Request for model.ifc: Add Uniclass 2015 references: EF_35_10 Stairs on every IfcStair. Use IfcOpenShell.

First a look at what the model holds.

```python
import ifcopenshell

model = ifcopenshell.open("model.ifc")
print(model.schema)
print("classifications:", [c.Name for c in model.by_type("IfcClassification")])
for ifc_class in ("IfcDoor", "IfcRoof", "IfcStair", "IfcWall", "IfcWindow"):
    print(ifc_class, len(model.by_type(ifc_class)))
```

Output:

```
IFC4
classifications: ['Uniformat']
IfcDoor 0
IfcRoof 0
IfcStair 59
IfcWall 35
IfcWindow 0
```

```python
import ifcopenshell
import ifcopenshell.api.classification

model = ifcopenshell.open("model.ifc")

system = ifcopenshell.api.classification.add_classification(model, classification="Uniclass 2015")

codes = {
    "IfcStair": ("EF_35_10", "Stairs"),
}
for ifc_class, (code, name) in codes.items():
    products = model.by_type(ifc_class)
    ifcopenshell.api.classification.add_reference(
        model, products=products, classification=system, identification=code, name=name
    )
    print(code, len(products))

model.write("model-out.ifc")
```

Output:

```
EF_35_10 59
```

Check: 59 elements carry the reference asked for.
